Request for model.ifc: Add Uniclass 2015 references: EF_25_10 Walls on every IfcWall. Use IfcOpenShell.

First a look at what the model holds.

```python
import ifcopenshell

model = ifcopenshell.open("model.ifc")
print(model.schema)
print("classifications:", [c.Name for c in model.by_type("IfcClassification")])
for ifc_class in ("IfcDoor", "IfcRoof", "IfcStair", "IfcWall", "IfcWindow"):
    print(ifc_class, len(model.by_type(ifc_class)))
```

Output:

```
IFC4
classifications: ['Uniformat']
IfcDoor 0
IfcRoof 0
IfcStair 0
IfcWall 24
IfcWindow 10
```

```python
import ifcopenshell
import ifcopenshell.api.classification

model = ifcopenshell.open("model.ifc")

system = ifcopenshell.api.classification.add_classification(model, classification="Uniclass 2015")

codes = {
    "IfcWall": ("EF_25_10", "Walls"),
}
for ifc_class, (code, name) in codes.items():
    products = model.by_type(ifc_class)
    ifcopenshell.api.classification.add_reference(
        model, products=products, classification=system, identification=code, name=name
    )
    print(code, len(products))

model.write("model_v2.ifc")
```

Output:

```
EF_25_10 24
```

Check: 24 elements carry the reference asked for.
